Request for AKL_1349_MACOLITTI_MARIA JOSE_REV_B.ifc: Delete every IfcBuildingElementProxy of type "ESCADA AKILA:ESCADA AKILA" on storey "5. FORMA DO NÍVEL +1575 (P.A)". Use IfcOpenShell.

First a look at what the model holds.

```python
import ifcopenshell
import ifcopenshell.util.element

model = ifcopenshell.open("AKL_1349_MACOLITTI_MARIA JOSE_REV_B.ifc")
print(model.schema)
storey = next(s for s in model.by_type("IfcBuildingStorey") if s.Name == "5. FORMA DO NÍVEL +1575 (P.A)")
proxies = [e for e in ifcopenshell.util.element.get_decomposition(storey) if e.is_a("IfcBuildingElementProxy")]
seen = {}
for e in proxies:
    element_type = ifcopenshell.util.element.get_type(e)
    name = element_type.Name if element_type not in (None, e) else None
    seen[name] = seen.get(name, 0) + 1
for name, count in sorted(seen.items(), key=str):
    print(count, "x", name)
```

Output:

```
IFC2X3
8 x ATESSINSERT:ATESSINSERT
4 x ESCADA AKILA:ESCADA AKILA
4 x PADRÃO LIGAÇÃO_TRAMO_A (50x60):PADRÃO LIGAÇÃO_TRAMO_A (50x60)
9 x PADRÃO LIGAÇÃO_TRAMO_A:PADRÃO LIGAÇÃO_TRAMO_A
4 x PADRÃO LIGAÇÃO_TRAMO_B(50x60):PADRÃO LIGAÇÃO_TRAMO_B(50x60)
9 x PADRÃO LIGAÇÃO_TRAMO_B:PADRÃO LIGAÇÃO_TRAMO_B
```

```python
import ifcopenshell
import ifcopenshell.api.root
import ifcopenshell.util.element

model = ifcopenshell.open("AKL_1349_MACOLITTI_MARIA JOSE_REV_B.ifc")

storey = next(s for s in model.by_type("IfcBuildingStorey") if s.Name == "5. FORMA DO NÍVEL +1575 (P.A)")
proxies = [e for e in ifcopenshell.util.element.get_decomposition(storey) if e.is_a("IfcBuildingElementProxy")]
targets = [e for e in proxies if (t := ifcopenshell.util.element.get_type(e)) not in (None, e) and t.Name == "ESCADA AKILA:ESCADA AKILA"]

for e in targets:
    ifcopenshell.api.root.remove_product(model, product=e)
print(len(targets), "removed")

model.write("AKL_1349_MACOLITTI_MARIA JOSE_REV_B_updated.ifc")
```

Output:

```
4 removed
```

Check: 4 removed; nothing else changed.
